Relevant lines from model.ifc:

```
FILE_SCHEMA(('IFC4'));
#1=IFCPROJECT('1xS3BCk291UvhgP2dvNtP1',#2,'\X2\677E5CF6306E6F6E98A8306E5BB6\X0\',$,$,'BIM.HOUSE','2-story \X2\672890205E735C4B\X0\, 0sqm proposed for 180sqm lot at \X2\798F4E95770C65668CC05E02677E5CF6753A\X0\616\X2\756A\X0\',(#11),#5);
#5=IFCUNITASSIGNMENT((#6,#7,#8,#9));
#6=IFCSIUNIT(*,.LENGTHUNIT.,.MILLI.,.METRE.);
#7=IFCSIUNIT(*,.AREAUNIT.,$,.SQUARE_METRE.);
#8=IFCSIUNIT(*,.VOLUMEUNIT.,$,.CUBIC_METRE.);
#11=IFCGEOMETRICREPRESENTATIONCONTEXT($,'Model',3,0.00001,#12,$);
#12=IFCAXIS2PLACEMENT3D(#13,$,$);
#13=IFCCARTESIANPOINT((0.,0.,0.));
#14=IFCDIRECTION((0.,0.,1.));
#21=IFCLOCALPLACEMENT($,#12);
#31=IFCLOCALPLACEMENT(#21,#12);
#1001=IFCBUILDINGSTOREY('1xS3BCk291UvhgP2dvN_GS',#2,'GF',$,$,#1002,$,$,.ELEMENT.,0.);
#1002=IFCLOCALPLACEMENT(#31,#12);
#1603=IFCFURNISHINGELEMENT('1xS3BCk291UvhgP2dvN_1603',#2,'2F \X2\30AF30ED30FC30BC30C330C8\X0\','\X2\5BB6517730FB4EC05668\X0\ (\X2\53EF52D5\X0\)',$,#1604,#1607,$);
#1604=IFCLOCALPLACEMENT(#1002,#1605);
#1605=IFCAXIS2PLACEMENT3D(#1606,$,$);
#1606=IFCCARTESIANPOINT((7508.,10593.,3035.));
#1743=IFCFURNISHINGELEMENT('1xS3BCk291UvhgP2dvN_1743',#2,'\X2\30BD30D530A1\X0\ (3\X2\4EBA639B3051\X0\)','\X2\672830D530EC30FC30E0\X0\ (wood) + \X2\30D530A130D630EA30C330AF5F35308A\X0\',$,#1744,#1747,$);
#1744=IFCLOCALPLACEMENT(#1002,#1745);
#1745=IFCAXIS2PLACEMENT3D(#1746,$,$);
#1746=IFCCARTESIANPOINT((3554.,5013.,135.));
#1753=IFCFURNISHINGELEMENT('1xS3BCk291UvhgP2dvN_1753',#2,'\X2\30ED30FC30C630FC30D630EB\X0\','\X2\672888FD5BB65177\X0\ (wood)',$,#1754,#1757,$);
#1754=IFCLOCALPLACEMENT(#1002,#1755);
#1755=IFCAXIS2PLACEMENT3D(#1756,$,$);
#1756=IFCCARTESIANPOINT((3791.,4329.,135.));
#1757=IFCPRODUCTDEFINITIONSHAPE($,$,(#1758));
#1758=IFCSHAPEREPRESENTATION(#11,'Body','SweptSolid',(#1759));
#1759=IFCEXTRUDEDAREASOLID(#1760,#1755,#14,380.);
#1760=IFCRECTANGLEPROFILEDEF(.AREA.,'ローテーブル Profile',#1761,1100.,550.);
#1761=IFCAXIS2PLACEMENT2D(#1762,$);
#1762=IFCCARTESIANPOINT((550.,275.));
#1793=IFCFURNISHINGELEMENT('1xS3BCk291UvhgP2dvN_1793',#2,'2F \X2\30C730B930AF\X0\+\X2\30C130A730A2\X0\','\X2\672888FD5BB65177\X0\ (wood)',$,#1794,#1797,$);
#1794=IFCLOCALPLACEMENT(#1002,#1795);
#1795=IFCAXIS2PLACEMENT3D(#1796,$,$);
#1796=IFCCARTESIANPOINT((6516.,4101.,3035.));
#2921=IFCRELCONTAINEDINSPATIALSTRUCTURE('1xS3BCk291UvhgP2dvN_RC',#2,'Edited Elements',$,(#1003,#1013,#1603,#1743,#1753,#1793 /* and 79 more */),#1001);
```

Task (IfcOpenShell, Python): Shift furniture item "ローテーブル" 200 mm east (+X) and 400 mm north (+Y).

```python
import ifcopenshell
import ifcopenshell.api.geometry
import ifcopenshell.util.placement
import ifcopenshell.util.unit

model = ifcopenshell.open("model.ifc")
unit_scale = ifcopenshell.util.unit.calculate_unit_scale(model)

item = model.by_id(1753)
matrix = ifcopenshell.util.placement.get_local_placement(item.ObjectPlacement)
matrix[0, 3] += 0.2 / unit_scale
matrix[1, 3] += 0.4 / unit_scale
ifcopenshell.api.geometry.edit_object_placement(model, product=item, matrix=matrix, is_si=False)

print(ifcopenshell.util.placement.get_local_placement(item.ObjectPlacement).round(3) + 0.0)

model.write("model-out.ifc")
```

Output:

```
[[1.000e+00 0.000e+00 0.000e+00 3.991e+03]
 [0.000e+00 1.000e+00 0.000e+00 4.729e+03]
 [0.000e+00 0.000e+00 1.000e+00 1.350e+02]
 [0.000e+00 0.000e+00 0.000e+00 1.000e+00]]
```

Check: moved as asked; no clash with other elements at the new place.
